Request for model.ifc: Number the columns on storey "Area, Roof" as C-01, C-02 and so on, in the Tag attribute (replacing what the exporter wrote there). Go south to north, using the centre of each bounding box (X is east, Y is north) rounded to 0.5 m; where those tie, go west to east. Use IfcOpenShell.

First a look at what the model holds.

```python
import ifcopenshell
import ifcopenshell.util.element
import ifcopenshell.util.placement

model = ifcopenshell.open("model.ifc")
print(model.schema)
storey = next(s for s in model.by_type("IfcBuildingStorey") if s.Name == "Area, Roof")
columns = [e for e in ifcopenshell.util.element.get_decomposition(storey) if e.is_a("IfcColumn")]
for e in sorted(columns, key=lambda e: e.id()):
    origin = ifcopenshell.util.placement.get_local_placement(e.ObjectPlacement)[:3, 3]
    print(e.id(), e.Tag, e.Name, origin.round(2) + 0.0, sep=" | ")
```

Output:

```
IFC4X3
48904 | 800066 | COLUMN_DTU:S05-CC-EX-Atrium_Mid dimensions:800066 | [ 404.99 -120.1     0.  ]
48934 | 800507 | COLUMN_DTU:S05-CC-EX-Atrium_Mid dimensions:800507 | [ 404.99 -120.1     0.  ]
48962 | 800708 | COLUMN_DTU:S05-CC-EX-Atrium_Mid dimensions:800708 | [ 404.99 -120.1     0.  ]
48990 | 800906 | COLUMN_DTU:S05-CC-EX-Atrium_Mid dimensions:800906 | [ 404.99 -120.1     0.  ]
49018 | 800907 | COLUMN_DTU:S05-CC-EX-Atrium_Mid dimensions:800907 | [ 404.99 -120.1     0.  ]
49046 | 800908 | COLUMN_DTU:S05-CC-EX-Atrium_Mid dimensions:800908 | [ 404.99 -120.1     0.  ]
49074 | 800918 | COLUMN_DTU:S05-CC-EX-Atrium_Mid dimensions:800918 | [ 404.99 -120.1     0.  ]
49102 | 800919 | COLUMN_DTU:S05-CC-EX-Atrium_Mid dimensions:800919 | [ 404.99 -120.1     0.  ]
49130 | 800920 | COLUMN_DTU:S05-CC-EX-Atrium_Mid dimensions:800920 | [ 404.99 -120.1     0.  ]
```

```python
import ifcopenshell
import ifcopenshell.geom
import ifcopenshell.util.element
import ifcopenshell.util.shape

model = ifcopenshell.open("model.ifc")
settings = ifcopenshell.geom.settings()
settings.set("use-world-coords", True)


def centre(element):
    shape = ifcopenshell.geom.create_shape(settings, element)
    return ifcopenshell.util.shape.get_bbox_centroid(shape.geometry)


storey = next(s for s in model.by_type("IfcBuildingStorey") if s.Name == "Area, Roof")
columns = [e for e in ifcopenshell.util.element.get_decomposition(storey) if e.is_a("IfcColumn")]

# Insertion points can sit at a corner or the storey origin, so sort by the geometry (in metres).
centres = {e: centre(e) for e in columns}
columns.sort(key=lambda e: (round(centres[e][1] / 0.5), centres[e][0]))

for i, e in enumerate(columns, start=1):
    number = f"C-{i:02d}"
    e.Tag = number
    print(e.id(), number)

model.write("model-out.ifc")
```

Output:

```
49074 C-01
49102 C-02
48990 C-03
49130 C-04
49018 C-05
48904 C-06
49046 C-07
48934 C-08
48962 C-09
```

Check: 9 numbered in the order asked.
